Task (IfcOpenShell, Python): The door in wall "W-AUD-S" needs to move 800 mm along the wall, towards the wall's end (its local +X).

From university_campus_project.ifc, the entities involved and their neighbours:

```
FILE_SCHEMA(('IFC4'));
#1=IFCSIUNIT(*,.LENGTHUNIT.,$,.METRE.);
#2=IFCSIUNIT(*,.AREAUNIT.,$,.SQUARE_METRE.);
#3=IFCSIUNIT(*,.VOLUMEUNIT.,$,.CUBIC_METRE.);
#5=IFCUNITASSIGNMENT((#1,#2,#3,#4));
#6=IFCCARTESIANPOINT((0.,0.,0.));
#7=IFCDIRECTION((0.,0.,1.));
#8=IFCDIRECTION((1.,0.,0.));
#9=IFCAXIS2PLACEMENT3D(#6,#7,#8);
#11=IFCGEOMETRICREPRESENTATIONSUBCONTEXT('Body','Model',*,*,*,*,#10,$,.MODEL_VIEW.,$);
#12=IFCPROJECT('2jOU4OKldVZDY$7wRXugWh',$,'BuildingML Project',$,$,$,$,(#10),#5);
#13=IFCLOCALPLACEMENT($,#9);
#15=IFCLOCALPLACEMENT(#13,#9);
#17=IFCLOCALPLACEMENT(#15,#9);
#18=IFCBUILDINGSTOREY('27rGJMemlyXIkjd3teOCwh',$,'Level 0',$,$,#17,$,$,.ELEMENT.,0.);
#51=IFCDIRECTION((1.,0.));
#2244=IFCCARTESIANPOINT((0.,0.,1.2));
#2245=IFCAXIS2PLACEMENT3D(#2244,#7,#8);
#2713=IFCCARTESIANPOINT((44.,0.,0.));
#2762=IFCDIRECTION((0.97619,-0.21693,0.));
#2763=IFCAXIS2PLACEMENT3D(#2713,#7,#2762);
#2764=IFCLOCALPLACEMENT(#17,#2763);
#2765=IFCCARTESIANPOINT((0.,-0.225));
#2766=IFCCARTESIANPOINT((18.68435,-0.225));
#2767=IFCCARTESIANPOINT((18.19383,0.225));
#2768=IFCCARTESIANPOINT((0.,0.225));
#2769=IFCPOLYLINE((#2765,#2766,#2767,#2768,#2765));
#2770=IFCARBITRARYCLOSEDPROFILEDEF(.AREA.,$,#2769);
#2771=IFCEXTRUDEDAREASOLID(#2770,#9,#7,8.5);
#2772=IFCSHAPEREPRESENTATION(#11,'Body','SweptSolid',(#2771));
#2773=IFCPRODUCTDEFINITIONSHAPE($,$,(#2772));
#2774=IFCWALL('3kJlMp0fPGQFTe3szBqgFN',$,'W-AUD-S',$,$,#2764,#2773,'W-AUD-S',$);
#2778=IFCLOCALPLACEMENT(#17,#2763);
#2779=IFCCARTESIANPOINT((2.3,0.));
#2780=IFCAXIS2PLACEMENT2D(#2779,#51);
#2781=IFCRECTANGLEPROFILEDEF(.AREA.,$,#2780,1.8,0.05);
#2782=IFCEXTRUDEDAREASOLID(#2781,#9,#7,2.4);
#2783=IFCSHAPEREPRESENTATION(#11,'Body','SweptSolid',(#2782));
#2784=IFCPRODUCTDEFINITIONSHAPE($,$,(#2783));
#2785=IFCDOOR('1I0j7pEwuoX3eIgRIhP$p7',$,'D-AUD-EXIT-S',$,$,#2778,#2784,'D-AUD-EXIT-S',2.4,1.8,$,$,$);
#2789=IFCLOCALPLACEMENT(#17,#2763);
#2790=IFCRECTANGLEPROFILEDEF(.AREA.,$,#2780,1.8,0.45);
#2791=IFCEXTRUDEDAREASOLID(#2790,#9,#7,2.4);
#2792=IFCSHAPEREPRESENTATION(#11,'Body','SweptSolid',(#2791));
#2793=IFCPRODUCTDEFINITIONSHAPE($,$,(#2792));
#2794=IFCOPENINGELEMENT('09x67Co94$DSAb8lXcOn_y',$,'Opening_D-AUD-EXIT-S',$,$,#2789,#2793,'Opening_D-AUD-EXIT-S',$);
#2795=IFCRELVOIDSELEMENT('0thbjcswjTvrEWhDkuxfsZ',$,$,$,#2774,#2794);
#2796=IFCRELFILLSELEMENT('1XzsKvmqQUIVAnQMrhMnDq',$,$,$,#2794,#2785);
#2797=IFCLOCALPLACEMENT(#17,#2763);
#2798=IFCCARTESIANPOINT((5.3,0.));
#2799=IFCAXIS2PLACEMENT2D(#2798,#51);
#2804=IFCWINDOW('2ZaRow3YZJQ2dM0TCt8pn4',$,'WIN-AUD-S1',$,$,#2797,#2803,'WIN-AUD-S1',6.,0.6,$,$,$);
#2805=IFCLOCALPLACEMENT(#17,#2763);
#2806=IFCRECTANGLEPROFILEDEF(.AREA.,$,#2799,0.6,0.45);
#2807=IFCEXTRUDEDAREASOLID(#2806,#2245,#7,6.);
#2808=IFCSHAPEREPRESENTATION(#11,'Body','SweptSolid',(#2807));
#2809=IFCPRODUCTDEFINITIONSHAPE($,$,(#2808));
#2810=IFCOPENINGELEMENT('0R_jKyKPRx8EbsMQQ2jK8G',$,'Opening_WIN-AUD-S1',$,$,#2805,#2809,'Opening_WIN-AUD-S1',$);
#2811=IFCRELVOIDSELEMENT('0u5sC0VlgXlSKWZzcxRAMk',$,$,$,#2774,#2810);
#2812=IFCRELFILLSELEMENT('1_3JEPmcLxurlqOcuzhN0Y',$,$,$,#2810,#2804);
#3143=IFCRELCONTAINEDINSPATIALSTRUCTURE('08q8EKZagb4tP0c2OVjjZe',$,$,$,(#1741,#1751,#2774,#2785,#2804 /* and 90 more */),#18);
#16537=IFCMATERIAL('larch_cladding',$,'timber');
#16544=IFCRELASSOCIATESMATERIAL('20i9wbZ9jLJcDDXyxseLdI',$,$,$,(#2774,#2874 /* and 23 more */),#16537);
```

```python
import ifcopenshell
import ifcopenshell.api.geometry
import ifcopenshell.util.placement
import ifcopenshell.util.unit

model = ifcopenshell.open("university_campus_project.ifc")
unit_scale = ifcopenshell.util.unit.calculate_unit_scale(model)

door = model.by_guid("1I0j7pEwuoX3eIgRIhP$p7")
opening = door.FillsVoids[0].RelatingOpeningElement
wall = opening.VoidsElements[0].RelatingBuildingElement

wall_matrix = ifcopenshell.util.placement.get_local_placement(wall.ObjectPlacement)
shift = wall_matrix[:3, 0] * 0.8 / unit_scale
before = ifcopenshell.util.placement.get_local_placement(door.ObjectPlacement)[:3, 3].copy()

# The door is not placed relative to its opening, so move both.
for product in (opening, door):
    matrix = ifcopenshell.util.placement.get_local_placement(product.ObjectPlacement)
    matrix[:3, 3] += shift
    ifcopenshell.api.geometry.edit_object_placement(model, product=product, matrix=matrix, is_si=False)

after = ifcopenshell.util.placement.get_local_placement(door.ObjectPlacement)[:3, 3]
print("door moved by", (after - before).round(3) + 0.0)

model.write("university_campus_project_rev.ifc")
```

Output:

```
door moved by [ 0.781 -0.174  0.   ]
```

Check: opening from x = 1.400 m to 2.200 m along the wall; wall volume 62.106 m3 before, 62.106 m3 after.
